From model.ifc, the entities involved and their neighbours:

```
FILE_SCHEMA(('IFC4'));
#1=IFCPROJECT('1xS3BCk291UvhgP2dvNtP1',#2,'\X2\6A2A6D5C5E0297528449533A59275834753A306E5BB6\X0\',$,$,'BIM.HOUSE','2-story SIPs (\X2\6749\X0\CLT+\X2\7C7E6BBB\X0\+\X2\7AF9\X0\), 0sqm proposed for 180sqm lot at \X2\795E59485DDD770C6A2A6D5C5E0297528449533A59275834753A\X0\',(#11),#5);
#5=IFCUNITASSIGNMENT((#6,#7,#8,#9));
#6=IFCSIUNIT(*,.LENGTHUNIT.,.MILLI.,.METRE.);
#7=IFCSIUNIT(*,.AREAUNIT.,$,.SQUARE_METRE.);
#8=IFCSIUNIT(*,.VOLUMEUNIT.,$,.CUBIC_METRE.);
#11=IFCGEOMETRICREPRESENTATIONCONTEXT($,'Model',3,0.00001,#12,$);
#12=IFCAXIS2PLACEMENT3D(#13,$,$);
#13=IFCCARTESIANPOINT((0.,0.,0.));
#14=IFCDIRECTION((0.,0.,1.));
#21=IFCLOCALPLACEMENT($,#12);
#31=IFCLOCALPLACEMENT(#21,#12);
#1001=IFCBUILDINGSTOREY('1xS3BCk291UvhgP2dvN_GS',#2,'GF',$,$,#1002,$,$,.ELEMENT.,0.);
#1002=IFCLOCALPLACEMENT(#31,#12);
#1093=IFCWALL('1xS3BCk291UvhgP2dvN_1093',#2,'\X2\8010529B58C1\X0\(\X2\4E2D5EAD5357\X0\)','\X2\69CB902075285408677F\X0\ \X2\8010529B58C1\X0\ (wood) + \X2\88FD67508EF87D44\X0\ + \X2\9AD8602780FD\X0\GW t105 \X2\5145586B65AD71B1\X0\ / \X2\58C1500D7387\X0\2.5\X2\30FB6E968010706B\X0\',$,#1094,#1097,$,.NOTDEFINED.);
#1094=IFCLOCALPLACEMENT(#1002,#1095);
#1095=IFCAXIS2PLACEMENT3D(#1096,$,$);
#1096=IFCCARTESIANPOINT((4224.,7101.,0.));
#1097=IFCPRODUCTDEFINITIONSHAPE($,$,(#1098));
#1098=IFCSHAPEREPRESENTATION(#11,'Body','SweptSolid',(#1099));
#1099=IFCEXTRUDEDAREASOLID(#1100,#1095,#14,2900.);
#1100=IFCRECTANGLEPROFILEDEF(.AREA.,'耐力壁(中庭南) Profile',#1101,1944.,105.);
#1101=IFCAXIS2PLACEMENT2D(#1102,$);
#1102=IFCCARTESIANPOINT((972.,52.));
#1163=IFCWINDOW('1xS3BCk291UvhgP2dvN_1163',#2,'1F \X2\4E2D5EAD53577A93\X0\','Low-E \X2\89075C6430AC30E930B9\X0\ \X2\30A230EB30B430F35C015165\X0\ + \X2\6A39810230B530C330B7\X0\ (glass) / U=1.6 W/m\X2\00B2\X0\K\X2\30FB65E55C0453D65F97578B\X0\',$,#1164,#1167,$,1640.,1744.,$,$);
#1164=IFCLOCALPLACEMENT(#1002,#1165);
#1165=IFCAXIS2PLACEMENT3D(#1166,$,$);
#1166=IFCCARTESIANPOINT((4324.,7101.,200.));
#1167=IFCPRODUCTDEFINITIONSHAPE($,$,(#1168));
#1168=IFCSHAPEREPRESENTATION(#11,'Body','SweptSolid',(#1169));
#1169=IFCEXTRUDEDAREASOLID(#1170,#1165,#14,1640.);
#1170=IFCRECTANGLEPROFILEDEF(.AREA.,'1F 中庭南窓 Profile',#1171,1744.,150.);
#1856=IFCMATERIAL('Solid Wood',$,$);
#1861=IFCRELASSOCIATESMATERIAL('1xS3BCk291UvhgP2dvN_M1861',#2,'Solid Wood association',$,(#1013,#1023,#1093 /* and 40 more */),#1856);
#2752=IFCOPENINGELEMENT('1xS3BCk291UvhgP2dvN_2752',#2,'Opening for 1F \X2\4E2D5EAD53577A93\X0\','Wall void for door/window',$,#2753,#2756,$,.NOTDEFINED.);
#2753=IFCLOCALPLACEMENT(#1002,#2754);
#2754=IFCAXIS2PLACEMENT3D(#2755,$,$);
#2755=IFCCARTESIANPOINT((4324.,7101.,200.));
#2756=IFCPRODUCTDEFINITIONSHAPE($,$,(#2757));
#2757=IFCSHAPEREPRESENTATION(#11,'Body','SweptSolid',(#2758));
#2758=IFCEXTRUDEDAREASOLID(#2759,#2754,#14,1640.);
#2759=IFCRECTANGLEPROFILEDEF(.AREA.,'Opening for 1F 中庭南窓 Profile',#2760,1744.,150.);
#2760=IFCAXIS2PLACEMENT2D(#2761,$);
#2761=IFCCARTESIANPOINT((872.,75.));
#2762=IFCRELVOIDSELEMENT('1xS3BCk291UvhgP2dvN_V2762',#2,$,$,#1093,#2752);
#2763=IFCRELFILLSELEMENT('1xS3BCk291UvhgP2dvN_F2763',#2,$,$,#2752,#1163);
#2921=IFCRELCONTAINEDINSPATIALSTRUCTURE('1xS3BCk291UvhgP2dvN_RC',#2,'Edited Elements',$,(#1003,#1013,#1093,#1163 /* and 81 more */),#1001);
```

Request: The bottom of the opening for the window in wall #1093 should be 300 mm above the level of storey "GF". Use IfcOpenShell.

```python
import numpy as np
import ifcopenshell
import ifcopenshell.api.geometry
import ifcopenshell.geom
import ifcopenshell.util.element
import ifcopenshell.util.placement
import ifcopenshell.util.shape
import ifcopenshell.util.unit

model = ifcopenshell.open("model.ifc")
unit_scale = ifcopenshell.util.unit.calculate_unit_scale(model)

window = model.by_id(1163)
opening = window.FillsVoids[0].RelatingOpeningElement
storey = ifcopenshell.util.element.get_container(window, ifc_class="IfcBuildingStorey")
level = ifcopenshell.util.placement.get_local_placement(storey.ObjectPlacement)[2, 3]

# The opening's origin need not be at the sill, so measure its lowest point.
shape = ifcopenshell.geom.create_shape(ifcopenshell.geom.settings(), opening)
bottom = ifcopenshell.util.shape.get_shape_bottom_elevation(shape, shape.geometry) / unit_scale
dz = level + 0.3 / unit_scale - bottom

shift = np.array([0.0, 0.0, dz])
# The window is not placed relative to its opening, so move both.
for product in (opening, window):
    matrix = ifcopenshell.util.placement.get_local_placement(product.ObjectPlacement)
    matrix[:3, 3] += shift
    ifcopenshell.api.geometry.edit_object_placement(model, product=product, matrix=matrix, is_si=False)

print(f"moved by {dz * unit_scale:+.3f} m")

model.write("model-out.ifc")
```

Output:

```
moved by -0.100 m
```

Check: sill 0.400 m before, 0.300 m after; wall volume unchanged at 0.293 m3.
